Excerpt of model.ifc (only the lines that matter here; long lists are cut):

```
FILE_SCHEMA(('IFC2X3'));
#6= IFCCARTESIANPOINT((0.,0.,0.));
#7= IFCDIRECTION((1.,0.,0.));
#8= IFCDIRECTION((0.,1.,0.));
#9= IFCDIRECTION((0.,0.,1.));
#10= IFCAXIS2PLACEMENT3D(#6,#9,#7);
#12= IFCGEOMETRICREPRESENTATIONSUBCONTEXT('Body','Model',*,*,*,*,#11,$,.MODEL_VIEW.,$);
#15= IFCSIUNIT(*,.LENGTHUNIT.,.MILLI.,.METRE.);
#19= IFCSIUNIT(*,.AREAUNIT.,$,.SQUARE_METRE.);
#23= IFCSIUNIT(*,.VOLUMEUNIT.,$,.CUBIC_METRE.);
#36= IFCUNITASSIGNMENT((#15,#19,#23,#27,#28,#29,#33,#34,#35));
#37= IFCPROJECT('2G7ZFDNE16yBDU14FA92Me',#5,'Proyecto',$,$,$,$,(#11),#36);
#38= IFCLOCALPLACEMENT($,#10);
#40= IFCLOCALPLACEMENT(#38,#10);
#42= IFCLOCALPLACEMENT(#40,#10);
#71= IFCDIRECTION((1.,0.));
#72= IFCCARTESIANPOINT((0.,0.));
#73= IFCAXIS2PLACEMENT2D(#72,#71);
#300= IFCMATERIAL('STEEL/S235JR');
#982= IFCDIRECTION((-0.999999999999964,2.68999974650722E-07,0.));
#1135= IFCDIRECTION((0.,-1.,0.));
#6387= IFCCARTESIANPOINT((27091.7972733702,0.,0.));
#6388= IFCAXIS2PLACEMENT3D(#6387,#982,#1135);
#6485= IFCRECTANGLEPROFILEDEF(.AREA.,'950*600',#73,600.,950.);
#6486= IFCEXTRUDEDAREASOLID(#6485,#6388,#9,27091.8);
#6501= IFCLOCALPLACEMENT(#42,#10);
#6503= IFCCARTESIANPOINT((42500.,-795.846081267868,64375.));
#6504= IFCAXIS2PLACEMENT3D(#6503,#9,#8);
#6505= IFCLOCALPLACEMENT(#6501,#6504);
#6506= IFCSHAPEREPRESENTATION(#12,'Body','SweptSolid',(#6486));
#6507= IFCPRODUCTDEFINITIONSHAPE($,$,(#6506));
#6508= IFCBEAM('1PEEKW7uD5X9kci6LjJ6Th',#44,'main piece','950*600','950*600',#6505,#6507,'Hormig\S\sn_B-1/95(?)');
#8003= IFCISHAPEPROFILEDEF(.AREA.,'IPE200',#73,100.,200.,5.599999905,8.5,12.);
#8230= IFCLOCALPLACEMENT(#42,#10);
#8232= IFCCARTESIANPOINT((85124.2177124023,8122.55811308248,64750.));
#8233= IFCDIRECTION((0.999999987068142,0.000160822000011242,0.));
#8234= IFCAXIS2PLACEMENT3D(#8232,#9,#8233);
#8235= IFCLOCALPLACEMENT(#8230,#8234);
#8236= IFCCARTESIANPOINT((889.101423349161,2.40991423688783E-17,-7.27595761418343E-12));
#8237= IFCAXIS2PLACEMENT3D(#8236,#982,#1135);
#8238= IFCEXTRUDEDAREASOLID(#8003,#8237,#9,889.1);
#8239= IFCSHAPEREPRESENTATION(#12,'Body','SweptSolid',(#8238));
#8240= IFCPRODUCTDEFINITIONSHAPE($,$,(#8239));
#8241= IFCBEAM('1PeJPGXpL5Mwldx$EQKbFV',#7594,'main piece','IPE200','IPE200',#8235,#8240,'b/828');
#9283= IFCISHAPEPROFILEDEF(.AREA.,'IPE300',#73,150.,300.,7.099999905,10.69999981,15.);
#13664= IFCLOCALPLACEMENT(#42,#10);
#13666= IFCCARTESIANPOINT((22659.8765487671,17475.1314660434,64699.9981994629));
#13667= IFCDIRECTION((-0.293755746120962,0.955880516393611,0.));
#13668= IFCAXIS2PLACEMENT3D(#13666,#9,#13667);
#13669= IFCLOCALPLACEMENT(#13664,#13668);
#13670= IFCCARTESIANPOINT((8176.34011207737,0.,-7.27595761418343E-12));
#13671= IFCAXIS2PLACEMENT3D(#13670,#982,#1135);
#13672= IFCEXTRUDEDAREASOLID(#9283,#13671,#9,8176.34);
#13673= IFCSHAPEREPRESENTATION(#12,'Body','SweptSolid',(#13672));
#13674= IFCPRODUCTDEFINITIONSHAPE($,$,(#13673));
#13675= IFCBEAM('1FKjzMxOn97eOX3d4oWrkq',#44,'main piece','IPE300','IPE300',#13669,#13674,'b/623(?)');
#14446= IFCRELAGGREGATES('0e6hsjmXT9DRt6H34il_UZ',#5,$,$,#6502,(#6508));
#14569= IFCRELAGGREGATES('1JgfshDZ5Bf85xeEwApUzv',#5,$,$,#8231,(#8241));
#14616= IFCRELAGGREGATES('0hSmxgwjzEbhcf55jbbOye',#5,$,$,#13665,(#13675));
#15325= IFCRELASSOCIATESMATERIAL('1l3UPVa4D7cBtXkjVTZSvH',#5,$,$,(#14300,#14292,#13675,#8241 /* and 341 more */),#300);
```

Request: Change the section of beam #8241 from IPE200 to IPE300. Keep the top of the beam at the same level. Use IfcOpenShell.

```python
import ifcopenshell
import ifcopenshell.util.element
import ifcopenshell.util.representation

model = ifcopenshell.open("model.ifc")

member = model.by_id(8241)
source = next(p for p in model.by_type("IfcIShapeProfileDef") if p.ProfileName == "IPE300")

body = ifcopenshell.util.representation.get_representation(member, "Model", "Body")
solid = body.Items[0]
old_profile = solid.SweptArea

# Copy the section's sizes but keep this member's own profile position.
profile = ifcopenshell.util.element.copy(model, source)
# Profiles are centred, so shift by half the change in depth to hold the top.
shift = (old_profile.OverallDepth - profile.OverallDepth) / 2
x, y = old_profile.Position.Location.Coordinates
up = (0.0, 1.0)  # upwards, in the solid's own plane
location = model.createIfcCartesianPoint((x + up[0] * shift, y + up[1] * shift))
profile.Position = model.createIfcAxis2Placement2D(location, old_profile.Position.RefDirection)
solid.SweptArea = profile
if not model.get_total_inverses(old_profile):
    ifcopenshell.util.element.remove_deep2(model, old_profile)
member.Description = member.Description.replace("IPE200", "IPE300")
member.ObjectType = member.ObjectType.replace("IPE200", "IPE300")

print(solid.SweptArea)

model.write("model_updated.ifc")
```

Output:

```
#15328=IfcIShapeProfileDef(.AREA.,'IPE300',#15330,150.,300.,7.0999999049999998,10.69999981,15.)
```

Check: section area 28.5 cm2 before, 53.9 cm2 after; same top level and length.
